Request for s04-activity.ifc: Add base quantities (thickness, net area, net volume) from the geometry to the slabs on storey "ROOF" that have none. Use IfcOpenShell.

First a look at what the model holds.

```python
import ifcopenshell
import ifcopenshell.util.element
import ifcopenshell.util.unit

model = ifcopenshell.open("s04-activity.ifc")
print(model.schema)
for unit_type in ("LENGTHUNIT", "AREAUNIT", "VOLUMEUNIT"):
    print(unit_type, ifcopenshell.util.unit.calculate_unit_scale(model, unit_type))
storey = next(s for s in model.by_type("IfcBuildingStorey") if s.Name == "ROOF")
slabs = [e for e in ifcopenshell.util.element.get_decomposition(storey) if e.is_a("IfcSlab")]
for e in sorted(slabs, key=lambda e: e.id()):
    print(e.id(), e.is_a(), e.Name, list(ifcopenshell.util.element.get_psets(e, qtos_only=True)), sep=" | ")
```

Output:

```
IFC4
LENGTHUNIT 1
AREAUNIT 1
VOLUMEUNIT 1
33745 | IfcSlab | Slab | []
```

```python
import ifcopenshell
import ifcopenshell.api.pset
import ifcopenshell.geom
import ifcopenshell.util.element
import ifcopenshell.util.shape
import ifcopenshell.util.unit

model = ifcopenshell.open("s04-activity.ifc")
unit_scale = ifcopenshell.util.unit.calculate_unit_scale(model)
area_scale = ifcopenshell.util.unit.calculate_unit_scale(model, "AREAUNIT")
volume_scale = ifcopenshell.util.unit.calculate_unit_scale(model, "VOLUMEUNIT")
settings = ifcopenshell.geom.settings()

storey = next(s for s in model.by_type("IfcBuildingStorey") if s.Name == "ROOF")
slabs = [e for e in ifcopenshell.util.element.get_decomposition(storey) if e.is_a("IfcSlab")]

for e in sorted(slabs, key=lambda e: e.id()):
    if ifcopenshell.util.element.get_psets(e, qtos_only=True, should_inherit=False):
        continue
    # Geometry comes back in metres, in the element's own axes.
    shape = ifcopenshell.geom.create_shape(settings, e)
    values = {
        "Width": ifcopenshell.util.shape.get_z(shape.geometry) / unit_scale,
        "NetArea": ifcopenshell.util.shape.get_footprint_area(shape.geometry) / area_scale,
        "NetVolume": ifcopenshell.util.shape.get_volume(shape.geometry) / volume_scale,
    }
    qto = ifcopenshell.api.pset.add_qto(model, product=e, name="Qto_SlabBaseQuantities")
    ifcopenshell.api.pset.edit_qto(model, qto=qto, properties=values)
    print(e.id(), {k: round(v, 3) for k, v in values.items()})

model.write("s04-activity_edited.ifc")
```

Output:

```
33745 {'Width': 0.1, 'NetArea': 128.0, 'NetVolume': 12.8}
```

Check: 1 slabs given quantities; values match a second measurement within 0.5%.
